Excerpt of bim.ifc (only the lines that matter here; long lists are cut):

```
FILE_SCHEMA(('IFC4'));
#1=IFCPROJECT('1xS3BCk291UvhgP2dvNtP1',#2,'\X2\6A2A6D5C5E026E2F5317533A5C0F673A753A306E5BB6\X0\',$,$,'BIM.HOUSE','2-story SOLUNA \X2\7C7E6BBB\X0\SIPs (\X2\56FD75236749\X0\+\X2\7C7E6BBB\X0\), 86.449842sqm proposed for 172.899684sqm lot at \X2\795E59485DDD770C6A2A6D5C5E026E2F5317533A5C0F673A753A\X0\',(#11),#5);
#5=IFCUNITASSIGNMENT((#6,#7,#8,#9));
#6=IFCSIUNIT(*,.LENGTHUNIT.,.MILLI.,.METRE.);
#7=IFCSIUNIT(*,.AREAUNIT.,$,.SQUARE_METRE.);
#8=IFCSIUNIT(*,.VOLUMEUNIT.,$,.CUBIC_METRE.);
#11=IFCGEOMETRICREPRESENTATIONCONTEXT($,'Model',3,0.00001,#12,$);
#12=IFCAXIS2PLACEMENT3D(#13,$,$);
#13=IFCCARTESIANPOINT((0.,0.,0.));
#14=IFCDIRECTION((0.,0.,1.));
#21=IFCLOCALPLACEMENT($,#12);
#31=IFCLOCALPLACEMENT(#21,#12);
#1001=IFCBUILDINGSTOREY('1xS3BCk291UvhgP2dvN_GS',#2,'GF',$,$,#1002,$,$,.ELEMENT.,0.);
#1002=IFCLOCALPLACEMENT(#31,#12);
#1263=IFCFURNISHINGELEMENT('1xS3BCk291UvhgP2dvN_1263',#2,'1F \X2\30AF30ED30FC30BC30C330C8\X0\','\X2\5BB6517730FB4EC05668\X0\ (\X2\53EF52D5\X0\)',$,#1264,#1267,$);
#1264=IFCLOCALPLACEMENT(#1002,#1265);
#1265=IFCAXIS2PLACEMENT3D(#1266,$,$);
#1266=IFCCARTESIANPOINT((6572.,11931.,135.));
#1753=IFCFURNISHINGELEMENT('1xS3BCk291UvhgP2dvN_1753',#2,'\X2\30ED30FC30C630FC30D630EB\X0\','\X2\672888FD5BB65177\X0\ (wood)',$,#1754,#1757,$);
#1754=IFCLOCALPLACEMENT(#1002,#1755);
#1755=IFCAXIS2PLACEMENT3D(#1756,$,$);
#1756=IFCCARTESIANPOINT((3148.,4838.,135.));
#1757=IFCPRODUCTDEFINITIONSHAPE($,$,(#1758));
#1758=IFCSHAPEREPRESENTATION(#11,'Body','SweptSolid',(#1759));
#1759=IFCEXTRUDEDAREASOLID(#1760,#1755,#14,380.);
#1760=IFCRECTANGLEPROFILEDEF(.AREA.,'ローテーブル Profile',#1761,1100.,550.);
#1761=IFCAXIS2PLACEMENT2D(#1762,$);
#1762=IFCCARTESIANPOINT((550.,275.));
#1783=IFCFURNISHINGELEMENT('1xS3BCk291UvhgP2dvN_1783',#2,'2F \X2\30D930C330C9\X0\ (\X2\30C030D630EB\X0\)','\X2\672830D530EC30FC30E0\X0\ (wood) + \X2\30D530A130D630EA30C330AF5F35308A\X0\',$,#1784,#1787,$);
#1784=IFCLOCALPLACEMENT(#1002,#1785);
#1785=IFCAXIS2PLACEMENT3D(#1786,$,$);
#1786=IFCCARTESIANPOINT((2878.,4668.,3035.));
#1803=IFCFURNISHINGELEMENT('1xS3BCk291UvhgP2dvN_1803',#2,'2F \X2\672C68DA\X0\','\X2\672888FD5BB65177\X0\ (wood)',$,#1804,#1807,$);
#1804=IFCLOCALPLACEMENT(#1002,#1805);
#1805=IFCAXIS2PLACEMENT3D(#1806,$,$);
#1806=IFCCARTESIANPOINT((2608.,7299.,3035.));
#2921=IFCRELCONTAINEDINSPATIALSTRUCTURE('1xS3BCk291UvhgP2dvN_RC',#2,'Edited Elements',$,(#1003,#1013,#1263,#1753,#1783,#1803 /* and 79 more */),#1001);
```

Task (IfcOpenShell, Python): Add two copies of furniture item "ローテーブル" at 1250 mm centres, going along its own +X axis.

```python
import ifcopenshell
import ifcopenshell.api.geometry
import ifcopenshell.api.root
import ifcopenshell.util.element
import ifcopenshell.util.placement
import ifcopenshell.util.unit

model = ifcopenshell.open("bim.ifc")
unit_scale = ifcopenshell.util.unit.calculate_unit_scale(model)


def reuse_history(source, copy):
    """copy_class also copies each property set's owner history, people and application; keep the originals."""
    for rel in copy.IsDefinedBy:
        if rel.is_a("IfcRelDefinesByProperties") and (history := rel.RelatingPropertyDefinition.OwnerHistory):
            rel.RelatingPropertyDefinition.OwnerHistory = source.OwnerHistory
            ifcopenshell.util.element.remove_deep2(model, history)


source = model.by_guid("1xS3BCk291UvhgP2dvN_1753")
base = ifcopenshell.util.placement.get_local_placement(source.ObjectPlacement)
step = base[:3, 0] * 1.25 / unit_scale

for i in range(1, 3):
    copy = ifcopenshell.api.root.copy_class(model, product=source)
    copy.Representation = ifcopenshell.util.element.copy_deep(
        model, source.Representation, exclude=["IfcGeometricRepresentationContext", "IfcRepresentationMap"]
    )
    reuse_history(source, copy)
    matrix = base.copy()
    matrix[:3, 3] += i * step
    print("added at", matrix[:3, 3].round(3) + 0.0)
    ifcopenshell.api.geometry.edit_object_placement(model, product=copy, matrix=matrix, is_si=False)

model.write("bim_edited.ifc")
```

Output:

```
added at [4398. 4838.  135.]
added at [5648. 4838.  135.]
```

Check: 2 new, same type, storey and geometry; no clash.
